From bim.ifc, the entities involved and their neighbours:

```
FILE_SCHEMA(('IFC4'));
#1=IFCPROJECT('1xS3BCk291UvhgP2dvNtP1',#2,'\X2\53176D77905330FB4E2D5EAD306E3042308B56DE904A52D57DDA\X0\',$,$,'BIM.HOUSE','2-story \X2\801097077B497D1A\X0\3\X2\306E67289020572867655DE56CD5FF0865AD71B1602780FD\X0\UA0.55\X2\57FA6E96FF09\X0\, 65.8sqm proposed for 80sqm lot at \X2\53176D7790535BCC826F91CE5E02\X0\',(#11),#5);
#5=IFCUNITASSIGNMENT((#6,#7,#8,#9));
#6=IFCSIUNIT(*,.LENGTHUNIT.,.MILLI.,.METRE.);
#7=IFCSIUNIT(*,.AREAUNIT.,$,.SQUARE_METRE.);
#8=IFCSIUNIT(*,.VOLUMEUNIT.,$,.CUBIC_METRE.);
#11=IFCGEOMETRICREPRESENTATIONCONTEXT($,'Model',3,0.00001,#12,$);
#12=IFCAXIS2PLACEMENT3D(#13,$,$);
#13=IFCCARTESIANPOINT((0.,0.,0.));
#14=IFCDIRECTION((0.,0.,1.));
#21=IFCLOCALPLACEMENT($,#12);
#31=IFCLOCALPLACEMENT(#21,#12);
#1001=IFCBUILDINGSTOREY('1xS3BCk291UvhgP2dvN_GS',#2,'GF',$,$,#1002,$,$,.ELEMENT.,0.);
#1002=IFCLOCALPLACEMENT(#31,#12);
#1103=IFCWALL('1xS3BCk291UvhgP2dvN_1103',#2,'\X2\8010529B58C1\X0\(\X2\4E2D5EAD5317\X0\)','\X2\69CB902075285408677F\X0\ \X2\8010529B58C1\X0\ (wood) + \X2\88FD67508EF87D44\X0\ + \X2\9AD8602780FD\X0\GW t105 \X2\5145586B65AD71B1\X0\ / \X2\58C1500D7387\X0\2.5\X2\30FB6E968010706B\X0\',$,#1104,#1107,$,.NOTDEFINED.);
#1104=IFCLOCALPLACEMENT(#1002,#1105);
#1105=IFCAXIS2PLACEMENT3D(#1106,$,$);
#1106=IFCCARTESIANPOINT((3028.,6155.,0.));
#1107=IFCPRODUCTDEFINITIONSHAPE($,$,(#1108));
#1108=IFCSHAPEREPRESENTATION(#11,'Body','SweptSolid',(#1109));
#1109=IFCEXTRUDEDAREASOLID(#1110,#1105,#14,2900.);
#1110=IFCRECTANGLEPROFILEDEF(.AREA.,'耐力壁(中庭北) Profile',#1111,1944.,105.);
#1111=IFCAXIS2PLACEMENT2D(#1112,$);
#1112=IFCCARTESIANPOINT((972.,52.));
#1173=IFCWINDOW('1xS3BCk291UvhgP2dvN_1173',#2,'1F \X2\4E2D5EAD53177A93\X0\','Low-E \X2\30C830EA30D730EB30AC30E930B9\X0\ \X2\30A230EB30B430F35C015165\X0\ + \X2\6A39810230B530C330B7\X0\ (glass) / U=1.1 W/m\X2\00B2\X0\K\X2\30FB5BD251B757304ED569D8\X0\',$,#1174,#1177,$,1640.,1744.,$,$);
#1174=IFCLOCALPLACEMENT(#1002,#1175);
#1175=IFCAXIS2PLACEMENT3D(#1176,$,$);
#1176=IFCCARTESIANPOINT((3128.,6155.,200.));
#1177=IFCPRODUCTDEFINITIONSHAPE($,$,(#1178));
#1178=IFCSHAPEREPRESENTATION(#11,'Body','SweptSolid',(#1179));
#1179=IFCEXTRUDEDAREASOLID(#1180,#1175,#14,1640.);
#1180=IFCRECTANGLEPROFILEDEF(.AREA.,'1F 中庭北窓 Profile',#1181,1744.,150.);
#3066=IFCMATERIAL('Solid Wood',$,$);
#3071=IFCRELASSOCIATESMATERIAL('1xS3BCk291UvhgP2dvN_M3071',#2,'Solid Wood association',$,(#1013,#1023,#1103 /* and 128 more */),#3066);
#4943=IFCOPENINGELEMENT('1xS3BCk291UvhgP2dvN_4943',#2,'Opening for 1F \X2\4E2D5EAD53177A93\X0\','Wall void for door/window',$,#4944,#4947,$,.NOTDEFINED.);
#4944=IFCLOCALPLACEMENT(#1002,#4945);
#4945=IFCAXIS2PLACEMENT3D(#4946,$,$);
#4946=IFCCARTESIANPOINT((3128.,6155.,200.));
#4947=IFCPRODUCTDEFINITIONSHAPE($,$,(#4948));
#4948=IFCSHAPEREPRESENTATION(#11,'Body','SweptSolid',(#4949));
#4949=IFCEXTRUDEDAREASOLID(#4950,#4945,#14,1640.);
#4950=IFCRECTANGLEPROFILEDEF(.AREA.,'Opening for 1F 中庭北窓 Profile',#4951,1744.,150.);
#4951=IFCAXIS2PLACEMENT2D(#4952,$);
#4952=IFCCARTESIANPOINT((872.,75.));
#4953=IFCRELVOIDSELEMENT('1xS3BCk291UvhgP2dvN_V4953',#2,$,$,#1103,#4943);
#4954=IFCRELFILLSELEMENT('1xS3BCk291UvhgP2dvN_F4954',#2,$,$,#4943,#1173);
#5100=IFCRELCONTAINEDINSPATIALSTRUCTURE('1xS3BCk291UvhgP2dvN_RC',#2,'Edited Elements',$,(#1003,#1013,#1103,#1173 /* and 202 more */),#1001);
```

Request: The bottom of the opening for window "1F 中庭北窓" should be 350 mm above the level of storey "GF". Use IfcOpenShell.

```python
import numpy as np
import ifcopenshell
import ifcopenshell.api.geometry
import ifcopenshell.geom
import ifcopenshell.util.element
import ifcopenshell.util.placement
import ifcopenshell.util.shape
import ifcopenshell.util.unit

model = ifcopenshell.open("bim.ifc")
unit_scale = ifcopenshell.util.unit.calculate_unit_scale(model)

window = model.by_id(1173)
opening = window.FillsVoids[0].RelatingOpeningElement
storey = ifcopenshell.util.element.get_container(window, ifc_class="IfcBuildingStorey")
level = ifcopenshell.util.placement.get_local_placement(storey.ObjectPlacement)[2, 3]

# The opening's origin need not be at the sill, so measure its lowest point.
shape = ifcopenshell.geom.create_shape(ifcopenshell.geom.settings(), opening)
bottom = ifcopenshell.util.shape.get_shape_bottom_elevation(shape, shape.geometry) / unit_scale
dz = level + 350.0 - bottom

shift = np.array([0.0, 0.0, dz])
# The window is not placed relative to its opening, so move both.
for product in (opening, window):
    matrix = ifcopenshell.util.placement.get_local_placement(product.ObjectPlacement)
    matrix[:3, 3] += shift
    ifcopenshell.api.geometry.edit_object_placement(model, product=product, matrix=matrix, is_si=False)

print(f"moved by {dz * unit_scale:+.3f} m")

model.write("bim_v2.ifc")
```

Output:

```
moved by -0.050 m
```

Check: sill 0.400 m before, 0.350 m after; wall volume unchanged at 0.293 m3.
